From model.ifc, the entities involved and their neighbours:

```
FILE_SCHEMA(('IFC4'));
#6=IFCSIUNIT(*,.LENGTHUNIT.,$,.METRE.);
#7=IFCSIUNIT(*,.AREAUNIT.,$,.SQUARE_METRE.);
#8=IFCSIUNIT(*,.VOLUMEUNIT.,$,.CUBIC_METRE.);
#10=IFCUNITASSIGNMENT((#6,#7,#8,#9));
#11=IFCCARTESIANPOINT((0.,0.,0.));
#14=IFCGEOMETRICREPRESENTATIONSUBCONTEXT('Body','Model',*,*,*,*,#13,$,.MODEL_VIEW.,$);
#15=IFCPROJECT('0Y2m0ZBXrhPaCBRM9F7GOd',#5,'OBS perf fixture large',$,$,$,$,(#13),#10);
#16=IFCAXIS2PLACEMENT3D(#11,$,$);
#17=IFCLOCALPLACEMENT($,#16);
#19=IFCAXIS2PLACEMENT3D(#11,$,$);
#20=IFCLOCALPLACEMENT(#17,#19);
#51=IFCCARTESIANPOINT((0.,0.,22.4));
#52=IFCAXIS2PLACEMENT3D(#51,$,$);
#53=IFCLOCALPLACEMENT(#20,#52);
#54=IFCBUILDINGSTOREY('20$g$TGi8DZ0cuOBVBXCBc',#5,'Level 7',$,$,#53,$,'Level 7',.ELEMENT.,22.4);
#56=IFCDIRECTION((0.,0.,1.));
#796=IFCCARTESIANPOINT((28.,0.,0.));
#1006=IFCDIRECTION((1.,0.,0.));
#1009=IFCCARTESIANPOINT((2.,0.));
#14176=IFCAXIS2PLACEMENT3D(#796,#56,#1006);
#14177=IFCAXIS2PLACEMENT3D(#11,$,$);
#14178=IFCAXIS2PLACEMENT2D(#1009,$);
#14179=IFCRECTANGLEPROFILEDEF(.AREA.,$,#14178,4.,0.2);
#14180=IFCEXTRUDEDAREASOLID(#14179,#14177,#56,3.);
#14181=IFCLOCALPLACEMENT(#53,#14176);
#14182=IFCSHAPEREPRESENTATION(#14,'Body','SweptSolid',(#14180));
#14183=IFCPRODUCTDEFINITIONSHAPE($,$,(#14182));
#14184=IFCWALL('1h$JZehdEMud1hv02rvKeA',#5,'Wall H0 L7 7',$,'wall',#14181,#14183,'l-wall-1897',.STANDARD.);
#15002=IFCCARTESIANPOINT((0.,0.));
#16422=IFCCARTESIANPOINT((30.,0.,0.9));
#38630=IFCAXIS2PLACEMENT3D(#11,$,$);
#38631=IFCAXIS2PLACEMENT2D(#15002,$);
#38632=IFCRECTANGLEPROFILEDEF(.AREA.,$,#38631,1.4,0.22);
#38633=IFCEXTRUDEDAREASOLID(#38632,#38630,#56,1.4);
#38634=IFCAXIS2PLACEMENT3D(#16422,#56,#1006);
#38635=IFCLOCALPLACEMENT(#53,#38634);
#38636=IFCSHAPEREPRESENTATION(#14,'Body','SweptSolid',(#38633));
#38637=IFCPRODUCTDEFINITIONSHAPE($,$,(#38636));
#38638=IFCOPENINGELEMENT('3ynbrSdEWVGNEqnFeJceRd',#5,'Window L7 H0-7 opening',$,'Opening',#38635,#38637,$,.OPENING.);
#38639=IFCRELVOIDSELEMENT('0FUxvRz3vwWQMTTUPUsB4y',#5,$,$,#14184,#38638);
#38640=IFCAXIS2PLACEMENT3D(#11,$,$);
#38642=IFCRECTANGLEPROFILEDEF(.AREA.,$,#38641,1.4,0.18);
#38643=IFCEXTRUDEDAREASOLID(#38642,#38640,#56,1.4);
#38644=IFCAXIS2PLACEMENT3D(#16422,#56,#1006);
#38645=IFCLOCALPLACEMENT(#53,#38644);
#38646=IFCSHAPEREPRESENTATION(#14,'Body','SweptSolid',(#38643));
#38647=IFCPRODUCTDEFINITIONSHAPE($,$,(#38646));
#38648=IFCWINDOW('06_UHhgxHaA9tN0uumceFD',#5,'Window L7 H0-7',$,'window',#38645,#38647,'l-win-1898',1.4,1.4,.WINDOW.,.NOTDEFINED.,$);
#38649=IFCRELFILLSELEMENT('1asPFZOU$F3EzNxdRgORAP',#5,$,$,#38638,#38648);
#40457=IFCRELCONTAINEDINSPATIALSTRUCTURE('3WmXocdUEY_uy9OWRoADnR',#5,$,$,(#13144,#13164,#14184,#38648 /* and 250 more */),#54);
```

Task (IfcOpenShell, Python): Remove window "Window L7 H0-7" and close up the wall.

```python
import ifcopenshell
import ifcopenshell.api.feature
import ifcopenshell.api.root
import ifcopenshell.geom
import ifcopenshell.util.shape

model = ifcopenshell.open("model.ifc")
settings = ifcopenshell.geom.settings()


def volume(element):
    """Net volume in cubic metres, openings subtracted."""
    shape = ifcopenshell.geom.create_shape(settings, element)
    return ifcopenshell.util.shape.get_volume(shape.geometry)


window = model.by_guid("06_UHhgxHaA9tN0uumceFD")
opening = window.FillsVoids[0].RelatingOpeningElement
wall = opening.VoidsElements[0].RelatingBuildingElement
before = volume(wall)

ifcopenshell.api.root.remove_product(model, product=window)
ifcopenshell.api.feature.remove_feature(model, feature=opening)

after = volume(wall)

print(f"wall volume {before:.3f} -> {after:.3f} m3")

model.write("model_edited.ifc")
```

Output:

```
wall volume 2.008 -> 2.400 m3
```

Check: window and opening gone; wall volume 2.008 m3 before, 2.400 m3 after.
